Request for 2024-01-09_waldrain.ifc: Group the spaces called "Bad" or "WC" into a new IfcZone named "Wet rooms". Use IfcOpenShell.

First a look at what the model holds.

```python
import ifcopenshell

model = ifcopenshell.open("2024-01-09_waldrain.ifc")
print(model.schema)
seen = {}
for space in model.by_type("IfcSpace"):
    seen[space.LongName] = seen.get(space.LongName, 0) + 1
for name, count in sorted(seen.items(), key=str):
    print(count, "x", name)
print("zones:", [z.Name for z in model.by_type("IfcZone")][:20])
```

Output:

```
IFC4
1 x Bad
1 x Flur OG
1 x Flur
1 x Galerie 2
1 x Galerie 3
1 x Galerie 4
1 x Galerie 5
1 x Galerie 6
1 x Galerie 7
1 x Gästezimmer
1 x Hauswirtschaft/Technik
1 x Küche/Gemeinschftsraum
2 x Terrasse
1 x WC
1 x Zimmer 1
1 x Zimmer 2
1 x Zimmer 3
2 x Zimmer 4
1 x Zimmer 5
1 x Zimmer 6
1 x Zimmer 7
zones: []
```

```python
import ifcopenshell
import ifcopenshell.api.group
import ifcopenshell.api.root

model = ifcopenshell.open("2024-01-09_waldrain.ifc")

names = {"Bad", "WC"}
spaces = [s for s in model.by_type("IfcSpace") if s.LongName in names]

zone = ifcopenshell.api.root.create_entity(model, ifc_class="IfcZone", name="Wet rooms")
ifcopenshell.api.group.assign_group(model, products=spaces, group=zone)
print(len(spaces), "spaces in", zone.Name)

model.write("2024-01-09_waldrain_v2.ifc")
```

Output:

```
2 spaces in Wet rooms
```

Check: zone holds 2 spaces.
